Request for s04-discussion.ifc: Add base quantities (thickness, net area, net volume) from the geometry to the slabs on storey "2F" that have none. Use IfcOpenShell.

First a look at what the model holds.

```python
import ifcopenshell
import ifcopenshell.util.element
import ifcopenshell.util.unit

model = ifcopenshell.open("s04-discussion.ifc")
print(model.schema)
for unit_type in ("LENGTHUNIT", "AREAUNIT", "VOLUMEUNIT"):
    print(unit_type, ifcopenshell.util.unit.calculate_unit_scale(model, unit_type))
storey = next(s for s in model.by_type("IfcBuildingStorey") if s.Name == "2F")
slabs = [e for e in ifcopenshell.util.element.get_decomposition(storey) if e.is_a("IfcSlab")]
for e in sorted(slabs, key=lambda e: e.id()):
    print(e.id(), e.is_a(), e.Name, list(ifcopenshell.util.element.get_psets(e, qtos_only=True)), sep=" | ")
```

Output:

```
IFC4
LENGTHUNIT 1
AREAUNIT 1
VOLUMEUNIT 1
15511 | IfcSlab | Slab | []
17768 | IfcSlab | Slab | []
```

```python
import ifcopenshell
import ifcopenshell.api.pset
import ifcopenshell.geom
import ifcopenshell.util.element
import ifcopenshell.util.shape
import ifcopenshell.util.unit

model = ifcopenshell.open("s04-discussion.ifc")
unit_scale = ifcopenshell.util.unit.calculate_unit_scale(model)
area_scale = ifcopenshell.util.unit.calculate_unit_scale(model, "AREAUNIT")
volume_scale = ifcopenshell.util.unit.calculate_unit_scale(model, "VOLUMEUNIT")
settings = ifcopenshell.geom.settings()

storey = next(s for s in model.by_type("IfcBuildingStorey") if s.Name == "2F")
slabs = [e for e in ifcopenshell.util.element.get_decomposition(storey) if e.is_a("IfcSlab")]

for e in sorted(slabs, key=lambda e: e.id()):
    if ifcopenshell.util.element.get_psets(e, qtos_only=True, should_inherit=False):
        continue
    # Geometry comes back in metres, in the element's own axes.
    shape = ifcopenshell.geom.create_shape(settings, e)
    values = {
        "Width": ifcopenshell.util.shape.get_z(shape.geometry) / unit_scale,
        "NetArea": ifcopenshell.util.shape.get_footprint_area(shape.geometry) / area_scale,
        "NetVolume": ifcopenshell.util.shape.get_volume(shape.geometry) / volume_scale,
    }
    qto = ifcopenshell.api.pset.add_qto(model, product=e, name="Qto_SlabBaseQuantities")
    ifcopenshell.api.pset.edit_qto(model, qto=qto, properties=values)
    print(e.id(), {k: round(v, 3) for k, v in values.items()})

model.write("s04-discussion_rev.ifc")
```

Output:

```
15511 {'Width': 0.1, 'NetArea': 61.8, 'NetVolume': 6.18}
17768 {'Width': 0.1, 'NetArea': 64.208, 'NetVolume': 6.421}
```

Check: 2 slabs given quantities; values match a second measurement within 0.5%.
